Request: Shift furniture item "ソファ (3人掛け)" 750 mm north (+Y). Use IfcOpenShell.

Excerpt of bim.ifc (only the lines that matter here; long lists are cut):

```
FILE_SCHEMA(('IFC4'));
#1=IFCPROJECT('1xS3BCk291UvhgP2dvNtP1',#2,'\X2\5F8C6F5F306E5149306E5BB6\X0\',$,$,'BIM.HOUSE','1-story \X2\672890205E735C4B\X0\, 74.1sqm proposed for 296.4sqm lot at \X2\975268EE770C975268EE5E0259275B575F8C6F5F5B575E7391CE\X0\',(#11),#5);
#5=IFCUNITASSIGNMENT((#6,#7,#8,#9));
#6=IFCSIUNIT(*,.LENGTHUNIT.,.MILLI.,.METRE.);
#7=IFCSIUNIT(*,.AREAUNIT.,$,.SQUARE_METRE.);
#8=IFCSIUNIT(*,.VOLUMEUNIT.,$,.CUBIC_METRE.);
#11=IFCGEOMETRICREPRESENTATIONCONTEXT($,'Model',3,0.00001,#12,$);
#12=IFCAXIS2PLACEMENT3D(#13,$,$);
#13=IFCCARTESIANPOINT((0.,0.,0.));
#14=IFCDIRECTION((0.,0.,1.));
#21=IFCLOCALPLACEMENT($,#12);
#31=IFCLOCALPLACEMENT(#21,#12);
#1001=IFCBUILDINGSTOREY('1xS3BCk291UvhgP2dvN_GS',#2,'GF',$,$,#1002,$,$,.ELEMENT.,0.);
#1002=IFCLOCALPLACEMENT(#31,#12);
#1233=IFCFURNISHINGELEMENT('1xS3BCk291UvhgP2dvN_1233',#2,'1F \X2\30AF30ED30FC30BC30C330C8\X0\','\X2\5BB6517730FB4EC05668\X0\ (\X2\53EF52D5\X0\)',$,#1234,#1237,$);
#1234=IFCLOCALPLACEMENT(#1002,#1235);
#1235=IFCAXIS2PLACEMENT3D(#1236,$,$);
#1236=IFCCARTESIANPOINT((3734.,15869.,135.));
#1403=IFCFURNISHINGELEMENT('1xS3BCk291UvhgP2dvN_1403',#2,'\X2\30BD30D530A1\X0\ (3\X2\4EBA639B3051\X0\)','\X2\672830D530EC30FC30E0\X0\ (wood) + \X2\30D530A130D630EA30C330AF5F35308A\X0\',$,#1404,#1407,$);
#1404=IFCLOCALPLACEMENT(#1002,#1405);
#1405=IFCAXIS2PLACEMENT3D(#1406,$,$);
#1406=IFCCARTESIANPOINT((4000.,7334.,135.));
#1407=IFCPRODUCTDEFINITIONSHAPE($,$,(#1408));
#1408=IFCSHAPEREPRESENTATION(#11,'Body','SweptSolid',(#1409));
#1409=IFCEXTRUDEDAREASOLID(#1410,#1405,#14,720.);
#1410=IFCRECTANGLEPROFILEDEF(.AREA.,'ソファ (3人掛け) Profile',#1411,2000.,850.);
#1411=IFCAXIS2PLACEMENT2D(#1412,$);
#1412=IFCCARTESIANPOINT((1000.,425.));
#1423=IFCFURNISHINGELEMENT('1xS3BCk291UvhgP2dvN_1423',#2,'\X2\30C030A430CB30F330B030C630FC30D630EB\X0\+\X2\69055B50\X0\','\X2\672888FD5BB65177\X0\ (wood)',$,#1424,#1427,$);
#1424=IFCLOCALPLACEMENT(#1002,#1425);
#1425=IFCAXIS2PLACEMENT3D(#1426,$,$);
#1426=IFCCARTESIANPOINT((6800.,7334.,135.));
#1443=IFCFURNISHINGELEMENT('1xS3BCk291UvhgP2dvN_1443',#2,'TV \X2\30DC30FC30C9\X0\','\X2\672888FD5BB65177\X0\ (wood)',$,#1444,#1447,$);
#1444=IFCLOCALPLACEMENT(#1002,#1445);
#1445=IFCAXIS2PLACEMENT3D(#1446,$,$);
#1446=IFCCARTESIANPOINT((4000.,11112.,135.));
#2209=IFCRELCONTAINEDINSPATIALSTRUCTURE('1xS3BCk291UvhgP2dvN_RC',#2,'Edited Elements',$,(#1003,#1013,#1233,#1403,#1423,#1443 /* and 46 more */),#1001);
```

```python
import ifcopenshell
import ifcopenshell.api.geometry
import ifcopenshell.util.placement

model = ifcopenshell.open("bim.ifc")

item = model.by_id(1403)
matrix = ifcopenshell.util.placement.get_local_placement(item.ObjectPlacement)
matrix[1, 3] += 750.0
ifcopenshell.api.geometry.edit_object_placement(model, product=item, matrix=matrix, is_si=False)

print(ifcopenshell.util.placement.get_local_placement(item.ObjectPlacement).round(3) + 0.0)

model.write("bim_rev.ifc")
```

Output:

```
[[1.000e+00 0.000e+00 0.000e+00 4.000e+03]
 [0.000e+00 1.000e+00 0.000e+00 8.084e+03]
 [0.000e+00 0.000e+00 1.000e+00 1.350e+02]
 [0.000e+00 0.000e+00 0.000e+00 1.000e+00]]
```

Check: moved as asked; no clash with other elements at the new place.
